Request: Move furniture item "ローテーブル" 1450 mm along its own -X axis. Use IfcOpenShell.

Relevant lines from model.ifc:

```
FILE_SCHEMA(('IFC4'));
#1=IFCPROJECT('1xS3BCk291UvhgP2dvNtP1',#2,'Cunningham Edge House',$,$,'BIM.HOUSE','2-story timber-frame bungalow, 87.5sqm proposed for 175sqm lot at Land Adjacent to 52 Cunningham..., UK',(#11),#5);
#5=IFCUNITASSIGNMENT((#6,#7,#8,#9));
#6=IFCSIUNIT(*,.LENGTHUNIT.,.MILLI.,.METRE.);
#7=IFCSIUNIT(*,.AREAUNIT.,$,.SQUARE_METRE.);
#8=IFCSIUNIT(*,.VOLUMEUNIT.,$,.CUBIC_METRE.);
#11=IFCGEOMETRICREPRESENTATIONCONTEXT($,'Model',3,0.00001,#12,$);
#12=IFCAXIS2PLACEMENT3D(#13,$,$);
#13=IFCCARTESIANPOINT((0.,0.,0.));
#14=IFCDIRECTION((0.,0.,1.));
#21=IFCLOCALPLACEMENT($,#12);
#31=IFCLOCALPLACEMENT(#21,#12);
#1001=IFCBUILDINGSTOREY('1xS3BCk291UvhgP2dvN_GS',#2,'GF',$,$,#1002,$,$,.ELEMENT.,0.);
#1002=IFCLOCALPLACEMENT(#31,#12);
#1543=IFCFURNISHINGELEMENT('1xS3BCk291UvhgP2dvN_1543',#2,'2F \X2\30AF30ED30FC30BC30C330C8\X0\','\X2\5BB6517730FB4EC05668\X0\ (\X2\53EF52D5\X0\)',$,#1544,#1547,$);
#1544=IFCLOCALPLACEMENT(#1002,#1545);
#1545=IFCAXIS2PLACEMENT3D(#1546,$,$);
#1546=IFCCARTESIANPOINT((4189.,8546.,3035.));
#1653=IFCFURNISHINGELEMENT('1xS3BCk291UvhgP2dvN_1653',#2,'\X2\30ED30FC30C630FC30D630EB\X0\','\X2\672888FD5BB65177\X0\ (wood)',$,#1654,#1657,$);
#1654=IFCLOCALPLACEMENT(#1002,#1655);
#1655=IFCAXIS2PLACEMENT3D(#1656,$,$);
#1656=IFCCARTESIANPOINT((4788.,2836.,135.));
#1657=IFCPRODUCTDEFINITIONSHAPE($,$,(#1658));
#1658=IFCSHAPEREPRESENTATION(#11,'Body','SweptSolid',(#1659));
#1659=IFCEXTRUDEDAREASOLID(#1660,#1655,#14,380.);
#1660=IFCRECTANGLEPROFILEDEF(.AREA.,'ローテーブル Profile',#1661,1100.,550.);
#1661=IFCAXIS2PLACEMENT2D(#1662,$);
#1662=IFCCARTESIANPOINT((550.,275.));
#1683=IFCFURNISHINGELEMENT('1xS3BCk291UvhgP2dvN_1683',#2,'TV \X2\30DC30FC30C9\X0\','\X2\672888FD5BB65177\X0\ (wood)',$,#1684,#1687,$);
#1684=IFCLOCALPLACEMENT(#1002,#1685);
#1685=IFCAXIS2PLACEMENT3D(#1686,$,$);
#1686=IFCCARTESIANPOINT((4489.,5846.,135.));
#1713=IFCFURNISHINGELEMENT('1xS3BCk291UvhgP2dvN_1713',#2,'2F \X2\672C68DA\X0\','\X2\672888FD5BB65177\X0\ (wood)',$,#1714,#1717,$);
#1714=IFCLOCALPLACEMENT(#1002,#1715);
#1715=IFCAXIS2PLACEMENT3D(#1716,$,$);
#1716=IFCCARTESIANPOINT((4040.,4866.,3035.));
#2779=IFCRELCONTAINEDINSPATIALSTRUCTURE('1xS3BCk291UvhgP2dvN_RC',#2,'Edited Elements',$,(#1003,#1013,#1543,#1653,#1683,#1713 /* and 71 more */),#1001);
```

```python
import ifcopenshell
import ifcopenshell.api.geometry
import ifcopenshell.util.placement
import ifcopenshell.util.unit

model = ifcopenshell.open("model.ifc")
unit_scale = ifcopenshell.util.unit.calculate_unit_scale(model)

item = model.by_guid("1xS3BCk291UvhgP2dvN_1653")
matrix = ifcopenshell.util.placement.get_local_placement(item.ObjectPlacement)
matrix[:3, 3] -= matrix[:3, 0] * 1.45 / unit_scale
ifcopenshell.api.geometry.edit_object_placement(model, product=item, matrix=matrix, is_si=False)

print(ifcopenshell.util.placement.get_local_placement(item.ObjectPlacement).round(3) + 0.0)

model.write("model_updated.ifc")
```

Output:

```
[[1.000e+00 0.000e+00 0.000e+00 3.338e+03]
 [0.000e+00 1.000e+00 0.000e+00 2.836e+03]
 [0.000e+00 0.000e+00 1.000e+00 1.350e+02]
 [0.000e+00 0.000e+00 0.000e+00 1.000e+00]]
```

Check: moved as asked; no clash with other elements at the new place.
